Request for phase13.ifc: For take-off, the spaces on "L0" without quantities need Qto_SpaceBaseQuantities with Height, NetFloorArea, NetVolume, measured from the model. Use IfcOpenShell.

First a look at what the model holds.

```python
import ifcopenshell
import ifcopenshell.util.element
import ifcopenshell.util.unit

model = ifcopenshell.open("phase13.ifc")
print(model.schema)
for unit_type in ("LENGTHUNIT", "AREAUNIT", "VOLUMEUNIT"):
    print(unit_type, ifcopenshell.util.unit.calculate_unit_scale(model, unit_type))
storey = next(s for s in model.by_type("IfcBuildingStorey") if s.Name == "L0")
spaces = [e for e in ifcopenshell.util.element.get_decomposition(storey) if e.is_a("IfcSpace")]
for e in sorted(spaces, key=lambda e: e.id()):
    print(e.id(), e.is_a(), e.Name, list(ifcopenshell.util.element.get_psets(e, qtos_only=True)), sep=" | ")
```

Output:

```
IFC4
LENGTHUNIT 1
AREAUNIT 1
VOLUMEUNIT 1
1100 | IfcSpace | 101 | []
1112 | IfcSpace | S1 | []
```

```python
import ifcopenshell
import ifcopenshell.api.pset
import ifcopenshell.geom
import ifcopenshell.util.element
import ifcopenshell.util.shape
import ifcopenshell.util.unit

model = ifcopenshell.open("phase13.ifc")
unit_scale = ifcopenshell.util.unit.calculate_unit_scale(model)
area_scale = ifcopenshell.util.unit.calculate_unit_scale(model, "AREAUNIT")
volume_scale = ifcopenshell.util.unit.calculate_unit_scale(model, "VOLUMEUNIT")
settings = ifcopenshell.geom.settings()

storey = next(s for s in model.by_type("IfcBuildingStorey") if s.Name == "L0")
spaces = [e for e in ifcopenshell.util.element.get_decomposition(storey) if e.is_a("IfcSpace")]

for e in sorted(spaces, key=lambda e: e.id()):
    if ifcopenshell.util.element.get_psets(e, qtos_only=True, should_inherit=False):
        continue
    # Geometry comes back in metres, in the element's own axes.
    shape = ifcopenshell.geom.create_shape(settings, e)
    values = {
        "Height": ifcopenshell.util.shape.get_z(shape.geometry) / unit_scale,
        "NetFloorArea": ifcopenshell.util.shape.get_footprint_area(shape.geometry) / area_scale,
        "NetVolume": ifcopenshell.util.shape.get_volume(shape.geometry) / volume_scale,
    }
    qto = ifcopenshell.api.pset.add_qto(model, product=e, name="Qto_SpaceBaseQuantities")
    ifcopenshell.api.pset.edit_qto(model, qto=qto, properties=values)
    print(e.id(), {k: round(v, 3) for k, v in values.items()})

model.write("phase13_updated.ifc")
```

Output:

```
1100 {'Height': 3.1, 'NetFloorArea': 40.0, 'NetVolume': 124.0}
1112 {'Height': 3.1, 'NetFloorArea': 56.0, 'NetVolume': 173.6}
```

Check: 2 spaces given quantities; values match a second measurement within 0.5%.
